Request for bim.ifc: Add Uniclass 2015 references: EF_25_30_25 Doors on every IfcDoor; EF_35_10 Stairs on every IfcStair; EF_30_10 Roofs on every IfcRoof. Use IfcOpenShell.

First a look at what the model holds.

```python
import ifcopenshell

model = ifcopenshell.open("bim.ifc")
print(model.schema)
print("classifications:", [c.Name for c in model.by_type("IfcClassification")])
for ifc_class in ("IfcDoor", "IfcRoof", "IfcStair", "IfcWall", "IfcWindow"):
    print(ifc_class, len(model.by_type(ifc_class)))
```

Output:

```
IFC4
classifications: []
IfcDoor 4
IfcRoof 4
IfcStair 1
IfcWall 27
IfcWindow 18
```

```python
import ifcopenshell
import ifcopenshell.api.classification

model = ifcopenshell.open("bim.ifc")

system = ifcopenshell.api.classification.add_classification(model, classification="Uniclass 2015")

codes = {
    "IfcDoor": ("EF_25_30_25", "Doors"),
    "IfcStair": ("EF_35_10", "Stairs"),
    "IfcRoof": ("EF_30_10", "Roofs"),
}
for ifc_class, (code, name) in codes.items():
    products = model.by_type(ifc_class)
    ifcopenshell.api.classification.add_reference(
        model, products=products, classification=system, identification=code, name=name
    )
    print(code, len(products))

model.write("bim-out.ifc")
```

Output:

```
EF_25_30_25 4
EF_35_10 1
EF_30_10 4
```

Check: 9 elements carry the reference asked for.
